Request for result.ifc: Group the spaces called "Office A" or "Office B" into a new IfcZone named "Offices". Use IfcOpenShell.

First a look at what the model holds.

```python
import ifcopenshell

model = ifcopenshell.open("result.ifc")
print(model.schema)
seen = {}
for space in model.by_type("IfcSpace"):
    seen[space.Name] = seen.get(space.Name, 0) + 1
for name, count in sorted(seen.items(), key=str):
    print(count, "x", name)
print("zones:", [z.Name for z in model.by_type("IfcZone")][:20])
```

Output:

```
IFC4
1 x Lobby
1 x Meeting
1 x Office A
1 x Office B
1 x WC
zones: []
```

```python
import ifcopenshell
import ifcopenshell.api.group
import ifcopenshell.api.root

model = ifcopenshell.open("result.ifc")

names = {"Office A", "Office B"}
spaces = [s for s in model.by_type("IfcSpace") if s.Name in names]

zone = ifcopenshell.api.root.create_entity(model, ifc_class="IfcZone", name="Offices")
ifcopenshell.api.group.assign_group(model, products=spaces, group=zone)
print(len(spaces), "spaces in", zone.Name)

model.write("result_edited.ifc")
```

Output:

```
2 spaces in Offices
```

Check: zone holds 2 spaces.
